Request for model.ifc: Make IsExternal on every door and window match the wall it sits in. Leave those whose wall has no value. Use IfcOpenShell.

First a look at what the model holds.

```python
import ifcopenshell
import ifcopenshell.util.element

model = ifcopenshell.open("model.ifc")
print(model.schema)
seen = {}
for e in model.by_type("IfcDoor") + model.by_type("IfcWindow"):
    if not e.FillsVoids:
        continue
    host = e.FillsVoids[0].RelatingOpeningElement.VoidsElements[0].RelatingBuildingElement
    own = ifcopenshell.util.element.get_pset(e, f"Pset_{e.is_a()[3:].removesuffix('StandardCase')}Common", "IsExternal")
    wall = ifcopenshell.util.element.get_pset(host, "Pset_WallCommon", "IsExternal")
    seen[e.is_a(), own, wall] = seen.get((e.is_a(), own, wall), 0) + 1
for (cls, own, wall), count in sorted(seen.items(), key=str):
    print(count, cls, "IsExternal:", own, "| host wall:", wall)
```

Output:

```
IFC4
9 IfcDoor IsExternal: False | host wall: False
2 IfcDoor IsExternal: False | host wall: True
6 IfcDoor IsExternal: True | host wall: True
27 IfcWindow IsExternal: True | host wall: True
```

```python
import ifcopenshell
import ifcopenshell.api.pset
import ifcopenshell.util.element

model = ifcopenshell.open("model.ifc")

count = 0
for ifc_class, pset_name in (("IfcDoor", "Pset_DoorCommon"), ("IfcWindow", "Pset_WindowCommon")):
    for e in model.by_type(ifc_class):
        if not e.FillsVoids:
            continue
        host = e.FillsVoids[0].RelatingOpeningElement.VoidsElements[0].RelatingBuildingElement
        external = ifcopenshell.util.element.get_pset(host, "Pset_WallCommon", "IsExternal")
        if external is None or ifcopenshell.util.element.get_pset(e, pset_name, "IsExternal") == external:
            continue
        pset = ifcopenshell.api.pset.add_pset(model, product=e, name=pset_name)
        ifcopenshell.api.pset.edit_pset(model, pset=pset, properties={"IsExternal": external})
        count += 1

print(count, "updated")

model.write("model-out.ifc")
```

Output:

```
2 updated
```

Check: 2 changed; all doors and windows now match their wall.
